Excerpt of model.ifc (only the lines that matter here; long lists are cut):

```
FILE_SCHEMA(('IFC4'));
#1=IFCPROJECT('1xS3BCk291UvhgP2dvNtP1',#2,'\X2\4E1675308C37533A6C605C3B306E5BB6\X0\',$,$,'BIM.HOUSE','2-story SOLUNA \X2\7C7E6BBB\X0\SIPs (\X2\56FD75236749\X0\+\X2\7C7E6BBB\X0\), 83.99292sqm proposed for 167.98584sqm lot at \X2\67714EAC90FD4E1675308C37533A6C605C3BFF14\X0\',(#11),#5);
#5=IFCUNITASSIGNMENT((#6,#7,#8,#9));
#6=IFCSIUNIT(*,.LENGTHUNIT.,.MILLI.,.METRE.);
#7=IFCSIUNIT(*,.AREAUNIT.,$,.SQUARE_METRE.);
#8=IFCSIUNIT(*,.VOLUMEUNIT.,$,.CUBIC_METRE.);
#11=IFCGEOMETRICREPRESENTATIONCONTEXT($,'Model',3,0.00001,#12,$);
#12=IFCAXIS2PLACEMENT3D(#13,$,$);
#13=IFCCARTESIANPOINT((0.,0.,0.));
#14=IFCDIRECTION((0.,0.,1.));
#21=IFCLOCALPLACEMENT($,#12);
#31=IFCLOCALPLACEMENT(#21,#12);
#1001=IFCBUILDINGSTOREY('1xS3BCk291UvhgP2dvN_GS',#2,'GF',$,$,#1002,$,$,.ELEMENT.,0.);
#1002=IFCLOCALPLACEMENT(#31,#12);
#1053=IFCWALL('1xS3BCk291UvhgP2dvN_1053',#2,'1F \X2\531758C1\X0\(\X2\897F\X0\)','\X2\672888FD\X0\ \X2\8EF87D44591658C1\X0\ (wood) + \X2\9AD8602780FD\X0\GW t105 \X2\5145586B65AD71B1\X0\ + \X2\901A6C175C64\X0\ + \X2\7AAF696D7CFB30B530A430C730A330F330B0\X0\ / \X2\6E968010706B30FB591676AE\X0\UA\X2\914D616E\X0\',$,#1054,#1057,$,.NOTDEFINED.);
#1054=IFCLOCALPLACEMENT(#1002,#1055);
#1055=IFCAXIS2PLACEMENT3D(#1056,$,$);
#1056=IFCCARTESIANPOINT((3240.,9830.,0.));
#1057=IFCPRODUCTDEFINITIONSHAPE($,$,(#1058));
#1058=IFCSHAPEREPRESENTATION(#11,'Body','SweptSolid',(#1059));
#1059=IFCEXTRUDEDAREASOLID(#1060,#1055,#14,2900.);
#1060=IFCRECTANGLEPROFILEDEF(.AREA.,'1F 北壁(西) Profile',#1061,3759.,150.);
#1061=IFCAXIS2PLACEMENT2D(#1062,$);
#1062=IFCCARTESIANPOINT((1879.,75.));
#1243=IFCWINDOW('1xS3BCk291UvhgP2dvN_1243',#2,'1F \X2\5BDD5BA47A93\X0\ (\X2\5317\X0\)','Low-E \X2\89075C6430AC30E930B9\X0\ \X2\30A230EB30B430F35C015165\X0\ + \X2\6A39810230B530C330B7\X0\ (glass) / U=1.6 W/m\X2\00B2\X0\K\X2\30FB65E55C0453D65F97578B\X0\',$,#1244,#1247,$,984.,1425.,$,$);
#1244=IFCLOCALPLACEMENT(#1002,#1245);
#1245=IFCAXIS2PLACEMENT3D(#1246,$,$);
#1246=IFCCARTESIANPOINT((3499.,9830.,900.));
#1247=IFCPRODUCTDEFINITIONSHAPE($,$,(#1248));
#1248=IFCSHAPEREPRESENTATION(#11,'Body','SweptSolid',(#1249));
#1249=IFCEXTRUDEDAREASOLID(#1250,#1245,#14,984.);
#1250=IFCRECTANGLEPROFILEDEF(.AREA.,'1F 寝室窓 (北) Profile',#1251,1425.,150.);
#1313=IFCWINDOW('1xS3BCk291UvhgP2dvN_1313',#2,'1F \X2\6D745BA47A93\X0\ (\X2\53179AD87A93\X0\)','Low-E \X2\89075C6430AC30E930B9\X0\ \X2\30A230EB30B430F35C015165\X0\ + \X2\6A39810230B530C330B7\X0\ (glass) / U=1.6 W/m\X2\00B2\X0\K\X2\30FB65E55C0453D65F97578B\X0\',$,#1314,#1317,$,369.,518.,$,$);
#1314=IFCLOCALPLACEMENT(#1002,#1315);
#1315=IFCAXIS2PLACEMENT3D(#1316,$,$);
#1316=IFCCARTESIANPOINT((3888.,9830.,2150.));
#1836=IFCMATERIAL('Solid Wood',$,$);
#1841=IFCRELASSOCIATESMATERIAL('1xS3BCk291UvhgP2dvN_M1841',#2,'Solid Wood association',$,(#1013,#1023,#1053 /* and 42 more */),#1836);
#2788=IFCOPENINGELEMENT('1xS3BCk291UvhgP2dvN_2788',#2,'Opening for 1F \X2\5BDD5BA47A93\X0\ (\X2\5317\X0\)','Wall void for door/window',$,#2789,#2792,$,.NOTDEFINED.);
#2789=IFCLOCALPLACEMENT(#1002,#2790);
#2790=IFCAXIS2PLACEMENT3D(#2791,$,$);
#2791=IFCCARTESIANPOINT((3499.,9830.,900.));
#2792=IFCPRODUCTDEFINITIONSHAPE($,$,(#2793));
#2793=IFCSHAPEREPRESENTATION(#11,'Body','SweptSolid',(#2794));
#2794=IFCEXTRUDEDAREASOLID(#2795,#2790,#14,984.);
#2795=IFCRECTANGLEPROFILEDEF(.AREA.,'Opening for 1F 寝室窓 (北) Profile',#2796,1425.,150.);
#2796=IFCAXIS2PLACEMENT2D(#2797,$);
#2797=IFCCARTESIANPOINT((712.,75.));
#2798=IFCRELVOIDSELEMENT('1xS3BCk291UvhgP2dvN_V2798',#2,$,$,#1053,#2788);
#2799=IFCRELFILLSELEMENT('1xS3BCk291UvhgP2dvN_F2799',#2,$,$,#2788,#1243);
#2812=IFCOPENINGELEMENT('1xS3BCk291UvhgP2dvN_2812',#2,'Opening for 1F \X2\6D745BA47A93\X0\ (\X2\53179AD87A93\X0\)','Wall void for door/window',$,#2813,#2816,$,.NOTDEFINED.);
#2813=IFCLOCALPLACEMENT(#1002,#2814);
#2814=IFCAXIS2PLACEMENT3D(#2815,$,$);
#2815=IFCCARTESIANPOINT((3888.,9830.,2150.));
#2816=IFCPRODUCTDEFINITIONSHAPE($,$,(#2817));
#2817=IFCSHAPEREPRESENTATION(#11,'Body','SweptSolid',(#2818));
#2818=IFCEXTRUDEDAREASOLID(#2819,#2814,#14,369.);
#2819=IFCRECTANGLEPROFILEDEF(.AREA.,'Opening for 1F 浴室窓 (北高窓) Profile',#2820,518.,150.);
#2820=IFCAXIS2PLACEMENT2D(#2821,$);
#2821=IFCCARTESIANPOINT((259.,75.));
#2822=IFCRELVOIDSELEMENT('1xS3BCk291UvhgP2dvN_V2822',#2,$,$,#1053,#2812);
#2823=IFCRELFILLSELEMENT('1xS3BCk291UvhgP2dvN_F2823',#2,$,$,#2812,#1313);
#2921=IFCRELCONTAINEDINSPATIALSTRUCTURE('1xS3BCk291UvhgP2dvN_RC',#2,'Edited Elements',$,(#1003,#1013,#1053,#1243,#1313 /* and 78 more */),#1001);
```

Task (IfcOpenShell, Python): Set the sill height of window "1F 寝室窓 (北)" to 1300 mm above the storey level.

```python
import numpy as np
import ifcopenshell
import ifcopenshell.api.geometry
import ifcopenshell.geom
import ifcopenshell.util.element
import ifcopenshell.util.placement
import ifcopenshell.util.shape
import ifcopenshell.util.unit

model = ifcopenshell.open("model.ifc")
unit_scale = ifcopenshell.util.unit.calculate_unit_scale(model)

window = model.by_id(1243)
opening = window.FillsVoids[0].RelatingOpeningElement
storey = ifcopenshell.util.element.get_container(window, ifc_class="IfcBuildingStorey")
level = ifcopenshell.util.placement.get_local_placement(storey.ObjectPlacement)[2, 3]

# The opening's origin need not be at the sill, so measure its lowest point.
shape = ifcopenshell.geom.create_shape(ifcopenshell.geom.settings(), opening)
bottom = ifcopenshell.util.shape.get_shape_bottom_elevation(shape, shape.geometry) / unit_scale
dz = level + 1.3 / unit_scale - bottom

shift = np.array([0.0, 0.0, dz])
# The window is not placed relative to its opening, so move both.
for product in (opening, window):
    matrix = ifcopenshell.util.placement.get_local_placement(product.ObjectPlacement)
    matrix[:3, 3] += shift
    ifcopenshell.api.geometry.edit_object_placement(model, product=product, matrix=matrix, is_si=False)

print(f"moved by {dz * unit_scale:+.3f} m")

model.write("model-out.ifc")
```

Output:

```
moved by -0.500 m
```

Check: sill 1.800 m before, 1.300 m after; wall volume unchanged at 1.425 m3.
